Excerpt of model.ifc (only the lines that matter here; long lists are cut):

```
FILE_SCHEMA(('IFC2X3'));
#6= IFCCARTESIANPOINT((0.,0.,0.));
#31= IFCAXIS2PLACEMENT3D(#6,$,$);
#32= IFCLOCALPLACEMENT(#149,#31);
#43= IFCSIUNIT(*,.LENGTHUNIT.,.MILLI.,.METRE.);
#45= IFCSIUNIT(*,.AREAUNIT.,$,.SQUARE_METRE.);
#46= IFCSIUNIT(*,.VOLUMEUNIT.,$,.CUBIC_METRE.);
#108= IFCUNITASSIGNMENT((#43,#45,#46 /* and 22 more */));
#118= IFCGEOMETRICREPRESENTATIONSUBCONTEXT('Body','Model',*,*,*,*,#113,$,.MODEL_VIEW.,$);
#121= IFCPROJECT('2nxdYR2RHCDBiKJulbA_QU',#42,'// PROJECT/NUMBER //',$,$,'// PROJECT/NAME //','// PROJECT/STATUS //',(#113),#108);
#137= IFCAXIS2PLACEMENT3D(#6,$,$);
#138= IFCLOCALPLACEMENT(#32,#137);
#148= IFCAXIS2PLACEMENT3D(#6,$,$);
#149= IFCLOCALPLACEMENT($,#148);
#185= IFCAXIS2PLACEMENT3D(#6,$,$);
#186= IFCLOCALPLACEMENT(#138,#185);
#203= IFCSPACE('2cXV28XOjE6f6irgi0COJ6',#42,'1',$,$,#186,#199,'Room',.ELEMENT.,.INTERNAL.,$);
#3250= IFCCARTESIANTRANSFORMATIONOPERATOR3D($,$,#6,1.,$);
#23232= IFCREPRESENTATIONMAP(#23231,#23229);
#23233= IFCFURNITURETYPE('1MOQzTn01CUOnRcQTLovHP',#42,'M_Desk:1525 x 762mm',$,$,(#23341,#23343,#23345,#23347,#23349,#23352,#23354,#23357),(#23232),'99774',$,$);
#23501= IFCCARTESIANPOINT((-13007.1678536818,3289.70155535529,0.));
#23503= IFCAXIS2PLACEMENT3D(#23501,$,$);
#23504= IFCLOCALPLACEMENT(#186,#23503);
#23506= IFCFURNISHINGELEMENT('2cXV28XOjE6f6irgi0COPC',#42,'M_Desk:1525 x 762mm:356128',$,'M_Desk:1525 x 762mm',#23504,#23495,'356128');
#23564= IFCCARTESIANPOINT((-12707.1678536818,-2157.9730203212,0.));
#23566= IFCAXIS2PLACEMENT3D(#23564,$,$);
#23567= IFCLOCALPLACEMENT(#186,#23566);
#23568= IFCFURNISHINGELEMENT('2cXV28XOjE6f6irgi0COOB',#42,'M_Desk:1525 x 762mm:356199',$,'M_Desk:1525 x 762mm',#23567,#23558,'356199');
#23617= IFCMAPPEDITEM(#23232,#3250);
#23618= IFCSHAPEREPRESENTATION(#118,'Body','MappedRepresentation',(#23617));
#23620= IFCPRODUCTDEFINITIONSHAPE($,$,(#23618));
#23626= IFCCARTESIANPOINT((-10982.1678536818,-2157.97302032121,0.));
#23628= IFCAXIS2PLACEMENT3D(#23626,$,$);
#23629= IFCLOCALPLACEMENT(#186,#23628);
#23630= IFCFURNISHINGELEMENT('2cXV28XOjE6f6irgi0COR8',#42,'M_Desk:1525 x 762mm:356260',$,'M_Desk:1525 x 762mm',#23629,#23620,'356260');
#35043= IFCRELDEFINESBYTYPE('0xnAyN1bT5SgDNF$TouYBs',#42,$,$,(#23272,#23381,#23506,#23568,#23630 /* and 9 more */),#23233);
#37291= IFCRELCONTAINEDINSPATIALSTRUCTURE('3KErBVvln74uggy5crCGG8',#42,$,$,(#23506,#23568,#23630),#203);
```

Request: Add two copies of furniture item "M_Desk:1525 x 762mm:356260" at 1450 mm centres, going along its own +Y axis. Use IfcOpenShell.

```python
import ifcopenshell
import ifcopenshell.api.geometry
import ifcopenshell.api.root
import ifcopenshell.util.element
import ifcopenshell.util.placement
import ifcopenshell.util.unit

model = ifcopenshell.open("model.ifc")
unit_scale = ifcopenshell.util.unit.calculate_unit_scale(model)


def reuse_history(source, copy):
    """copy_class also copies each property set's owner history, people and application; keep the originals."""
    for rel in copy.IsDefinedBy:
        if rel.is_a("IfcRelDefinesByProperties") and (history := rel.RelatingPropertyDefinition.OwnerHistory):
            rel.RelatingPropertyDefinition.OwnerHistory = source.OwnerHistory
            ifcopenshell.util.element.remove_deep2(model, history)


source = model.by_guid("2cXV28XOjE6f6irgi0COR8")
base = ifcopenshell.util.placement.get_local_placement(source.ObjectPlacement)
step = base[:3, 1] * 1.45 / unit_scale

for i in range(1, 3):
    copy = ifcopenshell.api.root.copy_class(model, product=source)
    copy.Representation = ifcopenshell.util.element.copy_deep(
        model, source.Representation, exclude=["IfcGeometricRepresentationContext", "IfcRepresentationMap"]
    )
    copy.Name = "M_Desk:1525 x 762mm"
    copy.Tag = None
    reuse_history(source, copy)
    matrix = base.copy()
    matrix[:3, 3] += i * step
    print("added at", matrix[:3, 3].round(3) + 0.0)
    ifcopenshell.api.geometry.edit_object_placement(model, product=copy, matrix=matrix, is_si=False)

model.write("model_rev.ifc")
```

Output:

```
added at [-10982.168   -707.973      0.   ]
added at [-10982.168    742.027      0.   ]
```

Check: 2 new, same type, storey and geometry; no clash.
